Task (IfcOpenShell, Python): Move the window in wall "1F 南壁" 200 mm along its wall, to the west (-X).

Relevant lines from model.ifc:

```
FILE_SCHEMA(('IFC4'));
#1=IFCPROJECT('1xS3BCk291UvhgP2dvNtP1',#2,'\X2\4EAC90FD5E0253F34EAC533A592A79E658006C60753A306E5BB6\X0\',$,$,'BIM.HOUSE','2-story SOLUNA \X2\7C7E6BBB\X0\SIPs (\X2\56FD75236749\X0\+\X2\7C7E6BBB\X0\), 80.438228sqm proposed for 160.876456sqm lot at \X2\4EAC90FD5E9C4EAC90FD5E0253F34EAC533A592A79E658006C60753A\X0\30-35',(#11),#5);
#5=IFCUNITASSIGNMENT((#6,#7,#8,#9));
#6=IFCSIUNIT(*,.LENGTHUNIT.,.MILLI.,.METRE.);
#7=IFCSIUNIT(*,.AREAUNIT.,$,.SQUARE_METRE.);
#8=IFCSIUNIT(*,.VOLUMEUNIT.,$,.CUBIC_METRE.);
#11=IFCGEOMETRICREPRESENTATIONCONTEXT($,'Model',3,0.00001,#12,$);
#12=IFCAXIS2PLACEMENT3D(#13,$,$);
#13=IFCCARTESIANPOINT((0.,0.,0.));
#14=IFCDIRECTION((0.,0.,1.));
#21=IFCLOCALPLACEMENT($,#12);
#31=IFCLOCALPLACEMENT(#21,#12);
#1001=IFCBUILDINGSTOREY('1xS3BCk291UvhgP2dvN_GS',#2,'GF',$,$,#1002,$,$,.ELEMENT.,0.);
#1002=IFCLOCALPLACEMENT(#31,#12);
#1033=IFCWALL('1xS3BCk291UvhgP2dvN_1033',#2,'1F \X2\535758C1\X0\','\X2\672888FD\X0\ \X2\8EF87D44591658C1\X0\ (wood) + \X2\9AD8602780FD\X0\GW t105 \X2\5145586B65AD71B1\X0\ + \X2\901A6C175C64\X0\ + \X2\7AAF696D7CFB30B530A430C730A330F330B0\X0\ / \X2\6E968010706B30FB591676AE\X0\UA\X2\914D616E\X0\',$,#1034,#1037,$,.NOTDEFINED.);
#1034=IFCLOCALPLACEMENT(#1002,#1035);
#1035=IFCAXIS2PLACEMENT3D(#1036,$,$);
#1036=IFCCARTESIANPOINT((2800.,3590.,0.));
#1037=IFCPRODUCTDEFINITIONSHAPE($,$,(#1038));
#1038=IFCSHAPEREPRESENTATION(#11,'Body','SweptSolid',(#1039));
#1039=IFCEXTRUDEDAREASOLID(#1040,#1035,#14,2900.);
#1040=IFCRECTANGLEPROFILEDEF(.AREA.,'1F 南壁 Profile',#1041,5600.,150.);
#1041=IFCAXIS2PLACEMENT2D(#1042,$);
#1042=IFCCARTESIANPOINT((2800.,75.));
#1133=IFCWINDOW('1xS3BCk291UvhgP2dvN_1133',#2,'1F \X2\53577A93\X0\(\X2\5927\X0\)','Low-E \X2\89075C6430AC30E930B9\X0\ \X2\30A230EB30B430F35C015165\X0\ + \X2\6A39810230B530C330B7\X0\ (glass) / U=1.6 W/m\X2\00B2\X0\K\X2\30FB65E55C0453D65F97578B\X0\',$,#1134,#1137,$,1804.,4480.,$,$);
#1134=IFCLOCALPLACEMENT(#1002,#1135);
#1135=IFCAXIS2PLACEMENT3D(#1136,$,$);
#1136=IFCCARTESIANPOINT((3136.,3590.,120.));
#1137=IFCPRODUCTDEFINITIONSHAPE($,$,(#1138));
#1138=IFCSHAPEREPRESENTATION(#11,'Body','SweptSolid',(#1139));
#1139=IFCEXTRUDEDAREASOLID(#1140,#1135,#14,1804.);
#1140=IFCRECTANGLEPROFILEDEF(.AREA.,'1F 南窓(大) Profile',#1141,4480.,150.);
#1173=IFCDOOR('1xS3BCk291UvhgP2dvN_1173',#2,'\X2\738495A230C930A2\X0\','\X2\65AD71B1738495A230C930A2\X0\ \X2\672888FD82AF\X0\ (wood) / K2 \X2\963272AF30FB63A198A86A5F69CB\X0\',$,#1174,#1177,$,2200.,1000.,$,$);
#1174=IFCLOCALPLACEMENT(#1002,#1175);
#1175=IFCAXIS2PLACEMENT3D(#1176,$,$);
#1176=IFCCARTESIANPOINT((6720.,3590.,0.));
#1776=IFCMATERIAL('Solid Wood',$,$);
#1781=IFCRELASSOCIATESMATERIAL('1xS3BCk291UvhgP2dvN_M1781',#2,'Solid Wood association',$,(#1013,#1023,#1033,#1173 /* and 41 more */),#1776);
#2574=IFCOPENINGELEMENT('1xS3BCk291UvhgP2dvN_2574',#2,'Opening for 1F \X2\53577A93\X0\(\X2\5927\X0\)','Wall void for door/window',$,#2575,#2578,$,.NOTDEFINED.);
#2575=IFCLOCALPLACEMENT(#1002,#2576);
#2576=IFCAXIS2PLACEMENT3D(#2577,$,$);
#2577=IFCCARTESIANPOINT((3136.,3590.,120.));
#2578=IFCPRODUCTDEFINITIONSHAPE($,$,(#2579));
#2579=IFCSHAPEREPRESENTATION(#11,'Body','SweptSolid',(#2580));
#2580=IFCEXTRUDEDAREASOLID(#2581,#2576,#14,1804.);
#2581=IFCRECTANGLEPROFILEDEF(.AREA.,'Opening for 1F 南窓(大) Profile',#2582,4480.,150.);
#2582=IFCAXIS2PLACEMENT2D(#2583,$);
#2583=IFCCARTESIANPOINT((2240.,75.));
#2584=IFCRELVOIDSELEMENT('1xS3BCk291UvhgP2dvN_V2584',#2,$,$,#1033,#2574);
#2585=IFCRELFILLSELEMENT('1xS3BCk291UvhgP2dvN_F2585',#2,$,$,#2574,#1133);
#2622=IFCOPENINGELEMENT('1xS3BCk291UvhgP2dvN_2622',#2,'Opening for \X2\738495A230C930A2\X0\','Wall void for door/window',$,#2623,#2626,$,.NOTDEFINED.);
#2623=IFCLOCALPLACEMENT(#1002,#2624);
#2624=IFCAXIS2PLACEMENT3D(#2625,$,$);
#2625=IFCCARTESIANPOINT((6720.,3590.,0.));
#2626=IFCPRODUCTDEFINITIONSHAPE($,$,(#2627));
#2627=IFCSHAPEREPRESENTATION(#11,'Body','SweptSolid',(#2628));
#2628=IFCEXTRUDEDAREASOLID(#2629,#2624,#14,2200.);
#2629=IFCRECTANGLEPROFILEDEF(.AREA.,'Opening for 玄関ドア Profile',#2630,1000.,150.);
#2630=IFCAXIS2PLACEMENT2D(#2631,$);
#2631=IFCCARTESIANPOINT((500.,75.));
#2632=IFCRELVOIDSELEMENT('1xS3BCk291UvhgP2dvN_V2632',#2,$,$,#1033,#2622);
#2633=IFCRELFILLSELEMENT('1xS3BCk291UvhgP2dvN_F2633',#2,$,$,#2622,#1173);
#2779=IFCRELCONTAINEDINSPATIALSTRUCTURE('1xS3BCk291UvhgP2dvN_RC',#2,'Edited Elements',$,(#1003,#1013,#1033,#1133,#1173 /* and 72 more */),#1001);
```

```python
import ifcopenshell
import ifcopenshell.api.geometry
import ifcopenshell.util.placement

model = ifcopenshell.open("model.ifc")

window = model.by_guid("1xS3BCk291UvhgP2dvN_1133")
opening = window.FillsVoids[0].RelatingOpeningElement
wall = opening.VoidsElements[0].RelatingBuildingElement

wall_matrix = ifcopenshell.util.placement.get_local_placement(wall.ObjectPlacement)
shift = wall_matrix[:3, 0] * -200.0
before = ifcopenshell.util.placement.get_local_placement(window.ObjectPlacement)[:3, 3].copy()

# The window is not placed relative to its opening, so move both.
for product in (opening, window):
    matrix = ifcopenshell.util.placement.get_local_placement(product.ObjectPlacement)
    matrix[:3, 3] += shift
    ifcopenshell.api.geometry.edit_object_placement(model, product=product, matrix=matrix, is_si=False)

after = ifcopenshell.util.placement.get_local_placement(window.ObjectPlacement)[:3, 3]
print("window moved by", (after - before).round(3) + 0.0)

model.write("model_edited.ifc")
```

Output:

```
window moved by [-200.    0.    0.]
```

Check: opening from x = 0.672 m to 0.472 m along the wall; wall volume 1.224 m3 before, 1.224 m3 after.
